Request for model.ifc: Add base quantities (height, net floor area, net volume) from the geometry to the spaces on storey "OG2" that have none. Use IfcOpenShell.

First a look at what the model holds.

```python
import ifcopenshell
import ifcopenshell.util.element
import ifcopenshell.util.unit

model = ifcopenshell.open("model.ifc")
print(model.schema)
for unit_type in ("LENGTHUNIT", "AREAUNIT", "VOLUMEUNIT"):
    print(unit_type, ifcopenshell.util.unit.calculate_unit_scale(model, unit_type))
storey = next(s for s in model.by_type("IfcBuildingStorey") if s.Name == "OG2")
spaces = [e for e in ifcopenshell.util.element.get_decomposition(storey) if e.is_a("IfcSpace")]
for e in sorted(spaces, key=lambda e: e.id()):
    print(e.id(), e.is_a(), e.Name, list(ifcopenshell.util.element.get_psets(e, qtos_only=True)), sep=" | ")
```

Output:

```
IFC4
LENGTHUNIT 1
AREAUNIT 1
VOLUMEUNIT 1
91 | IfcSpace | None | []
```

```python
import ifcopenshell
import ifcopenshell.api.pset
import ifcopenshell.geom
import ifcopenshell.util.element
import ifcopenshell.util.shape
import ifcopenshell.util.unit

model = ifcopenshell.open("model.ifc")
unit_scale = ifcopenshell.util.unit.calculate_unit_scale(model)
area_scale = ifcopenshell.util.unit.calculate_unit_scale(model, "AREAUNIT")
volume_scale = ifcopenshell.util.unit.calculate_unit_scale(model, "VOLUMEUNIT")
settings = ifcopenshell.geom.settings()

storey = next(s for s in model.by_type("IfcBuildingStorey") if s.Name == "OG2")
spaces = [e for e in ifcopenshell.util.element.get_decomposition(storey) if e.is_a("IfcSpace")]

for e in sorted(spaces, key=lambda e: e.id()):
    if ifcopenshell.util.element.get_psets(e, qtos_only=True, should_inherit=False):
        continue
    # Geometry comes back in metres, in the element's own axes.
    shape = ifcopenshell.geom.create_shape(settings, e)
    values = {
        "Height": ifcopenshell.util.shape.get_z(shape.geometry) / unit_scale,
        "NetFloorArea": ifcopenshell.util.shape.get_footprint_area(shape.geometry) / area_scale,
        "NetVolume": ifcopenshell.util.shape.get_volume(shape.geometry) / volume_scale,
    }
    qto = ifcopenshell.api.pset.add_qto(model, product=e, name="Qto_SpaceBaseQuantities")
    ifcopenshell.api.pset.edit_qto(model, qto=qto, properties=values)
    print(e.id(), {k: round(v, 3) for k, v in values.items()})

model.write("model_rev.ifc")
```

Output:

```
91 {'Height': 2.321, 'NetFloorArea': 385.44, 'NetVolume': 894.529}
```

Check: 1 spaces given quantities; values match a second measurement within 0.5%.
